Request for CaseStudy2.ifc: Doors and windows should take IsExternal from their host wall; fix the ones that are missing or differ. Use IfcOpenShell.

First a look at what the model holds.

```python
import ifcopenshell
import ifcopenshell.util.element

model = ifcopenshell.open("CaseStudy2.ifc")
print(model.schema)
seen = {}
for e in model.by_type("IfcDoor") + model.by_type("IfcWindow"):
    if not e.FillsVoids:
        continue
    host = e.FillsVoids[0].RelatingOpeningElement.VoidsElements[0].RelatingBuildingElement
    own = ifcopenshell.util.element.get_pset(e, f"Pset_{e.is_a()[3:].removesuffix('StandardCase')}Common", "IsExternal")
    wall = ifcopenshell.util.element.get_pset(host, "Pset_WallCommon", "IsExternal")
    seen[e.is_a(), own, wall] = seen.get((e.is_a(), own, wall), 0) + 1
for (cls, own, wall), count in sorted(seen.items(), key=str):
    print(count, cls, "IsExternal:", own, "| host wall:", wall)
```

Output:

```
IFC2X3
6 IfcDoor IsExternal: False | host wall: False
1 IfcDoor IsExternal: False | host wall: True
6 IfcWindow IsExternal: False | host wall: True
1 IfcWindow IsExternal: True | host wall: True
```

```python
import ifcopenshell
import ifcopenshell.api.pset
import ifcopenshell.util.element

model = ifcopenshell.open("CaseStudy2.ifc")

count = 0
for ifc_class, pset_name in (("IfcDoor", "Pset_DoorCommon"), ("IfcWindow", "Pset_WindowCommon")):
    for e in model.by_type(ifc_class):
        if not e.FillsVoids:
            continue
        host = e.FillsVoids[0].RelatingOpeningElement.VoidsElements[0].RelatingBuildingElement
        external = ifcopenshell.util.element.get_pset(host, "Pset_WallCommon", "IsExternal")
        if external is None or ifcopenshell.util.element.get_pset(e, pset_name, "IsExternal") == external:
            continue
        pset = ifcopenshell.api.pset.add_pset(model, product=e, name=pset_name)
        ifcopenshell.api.pset.edit_pset(model, pset=pset, properties={"IsExternal": external})
        count += 1

print(count, "updated")

model.write("CaseStudy2_edited.ifc")
```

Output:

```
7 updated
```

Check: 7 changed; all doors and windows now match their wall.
